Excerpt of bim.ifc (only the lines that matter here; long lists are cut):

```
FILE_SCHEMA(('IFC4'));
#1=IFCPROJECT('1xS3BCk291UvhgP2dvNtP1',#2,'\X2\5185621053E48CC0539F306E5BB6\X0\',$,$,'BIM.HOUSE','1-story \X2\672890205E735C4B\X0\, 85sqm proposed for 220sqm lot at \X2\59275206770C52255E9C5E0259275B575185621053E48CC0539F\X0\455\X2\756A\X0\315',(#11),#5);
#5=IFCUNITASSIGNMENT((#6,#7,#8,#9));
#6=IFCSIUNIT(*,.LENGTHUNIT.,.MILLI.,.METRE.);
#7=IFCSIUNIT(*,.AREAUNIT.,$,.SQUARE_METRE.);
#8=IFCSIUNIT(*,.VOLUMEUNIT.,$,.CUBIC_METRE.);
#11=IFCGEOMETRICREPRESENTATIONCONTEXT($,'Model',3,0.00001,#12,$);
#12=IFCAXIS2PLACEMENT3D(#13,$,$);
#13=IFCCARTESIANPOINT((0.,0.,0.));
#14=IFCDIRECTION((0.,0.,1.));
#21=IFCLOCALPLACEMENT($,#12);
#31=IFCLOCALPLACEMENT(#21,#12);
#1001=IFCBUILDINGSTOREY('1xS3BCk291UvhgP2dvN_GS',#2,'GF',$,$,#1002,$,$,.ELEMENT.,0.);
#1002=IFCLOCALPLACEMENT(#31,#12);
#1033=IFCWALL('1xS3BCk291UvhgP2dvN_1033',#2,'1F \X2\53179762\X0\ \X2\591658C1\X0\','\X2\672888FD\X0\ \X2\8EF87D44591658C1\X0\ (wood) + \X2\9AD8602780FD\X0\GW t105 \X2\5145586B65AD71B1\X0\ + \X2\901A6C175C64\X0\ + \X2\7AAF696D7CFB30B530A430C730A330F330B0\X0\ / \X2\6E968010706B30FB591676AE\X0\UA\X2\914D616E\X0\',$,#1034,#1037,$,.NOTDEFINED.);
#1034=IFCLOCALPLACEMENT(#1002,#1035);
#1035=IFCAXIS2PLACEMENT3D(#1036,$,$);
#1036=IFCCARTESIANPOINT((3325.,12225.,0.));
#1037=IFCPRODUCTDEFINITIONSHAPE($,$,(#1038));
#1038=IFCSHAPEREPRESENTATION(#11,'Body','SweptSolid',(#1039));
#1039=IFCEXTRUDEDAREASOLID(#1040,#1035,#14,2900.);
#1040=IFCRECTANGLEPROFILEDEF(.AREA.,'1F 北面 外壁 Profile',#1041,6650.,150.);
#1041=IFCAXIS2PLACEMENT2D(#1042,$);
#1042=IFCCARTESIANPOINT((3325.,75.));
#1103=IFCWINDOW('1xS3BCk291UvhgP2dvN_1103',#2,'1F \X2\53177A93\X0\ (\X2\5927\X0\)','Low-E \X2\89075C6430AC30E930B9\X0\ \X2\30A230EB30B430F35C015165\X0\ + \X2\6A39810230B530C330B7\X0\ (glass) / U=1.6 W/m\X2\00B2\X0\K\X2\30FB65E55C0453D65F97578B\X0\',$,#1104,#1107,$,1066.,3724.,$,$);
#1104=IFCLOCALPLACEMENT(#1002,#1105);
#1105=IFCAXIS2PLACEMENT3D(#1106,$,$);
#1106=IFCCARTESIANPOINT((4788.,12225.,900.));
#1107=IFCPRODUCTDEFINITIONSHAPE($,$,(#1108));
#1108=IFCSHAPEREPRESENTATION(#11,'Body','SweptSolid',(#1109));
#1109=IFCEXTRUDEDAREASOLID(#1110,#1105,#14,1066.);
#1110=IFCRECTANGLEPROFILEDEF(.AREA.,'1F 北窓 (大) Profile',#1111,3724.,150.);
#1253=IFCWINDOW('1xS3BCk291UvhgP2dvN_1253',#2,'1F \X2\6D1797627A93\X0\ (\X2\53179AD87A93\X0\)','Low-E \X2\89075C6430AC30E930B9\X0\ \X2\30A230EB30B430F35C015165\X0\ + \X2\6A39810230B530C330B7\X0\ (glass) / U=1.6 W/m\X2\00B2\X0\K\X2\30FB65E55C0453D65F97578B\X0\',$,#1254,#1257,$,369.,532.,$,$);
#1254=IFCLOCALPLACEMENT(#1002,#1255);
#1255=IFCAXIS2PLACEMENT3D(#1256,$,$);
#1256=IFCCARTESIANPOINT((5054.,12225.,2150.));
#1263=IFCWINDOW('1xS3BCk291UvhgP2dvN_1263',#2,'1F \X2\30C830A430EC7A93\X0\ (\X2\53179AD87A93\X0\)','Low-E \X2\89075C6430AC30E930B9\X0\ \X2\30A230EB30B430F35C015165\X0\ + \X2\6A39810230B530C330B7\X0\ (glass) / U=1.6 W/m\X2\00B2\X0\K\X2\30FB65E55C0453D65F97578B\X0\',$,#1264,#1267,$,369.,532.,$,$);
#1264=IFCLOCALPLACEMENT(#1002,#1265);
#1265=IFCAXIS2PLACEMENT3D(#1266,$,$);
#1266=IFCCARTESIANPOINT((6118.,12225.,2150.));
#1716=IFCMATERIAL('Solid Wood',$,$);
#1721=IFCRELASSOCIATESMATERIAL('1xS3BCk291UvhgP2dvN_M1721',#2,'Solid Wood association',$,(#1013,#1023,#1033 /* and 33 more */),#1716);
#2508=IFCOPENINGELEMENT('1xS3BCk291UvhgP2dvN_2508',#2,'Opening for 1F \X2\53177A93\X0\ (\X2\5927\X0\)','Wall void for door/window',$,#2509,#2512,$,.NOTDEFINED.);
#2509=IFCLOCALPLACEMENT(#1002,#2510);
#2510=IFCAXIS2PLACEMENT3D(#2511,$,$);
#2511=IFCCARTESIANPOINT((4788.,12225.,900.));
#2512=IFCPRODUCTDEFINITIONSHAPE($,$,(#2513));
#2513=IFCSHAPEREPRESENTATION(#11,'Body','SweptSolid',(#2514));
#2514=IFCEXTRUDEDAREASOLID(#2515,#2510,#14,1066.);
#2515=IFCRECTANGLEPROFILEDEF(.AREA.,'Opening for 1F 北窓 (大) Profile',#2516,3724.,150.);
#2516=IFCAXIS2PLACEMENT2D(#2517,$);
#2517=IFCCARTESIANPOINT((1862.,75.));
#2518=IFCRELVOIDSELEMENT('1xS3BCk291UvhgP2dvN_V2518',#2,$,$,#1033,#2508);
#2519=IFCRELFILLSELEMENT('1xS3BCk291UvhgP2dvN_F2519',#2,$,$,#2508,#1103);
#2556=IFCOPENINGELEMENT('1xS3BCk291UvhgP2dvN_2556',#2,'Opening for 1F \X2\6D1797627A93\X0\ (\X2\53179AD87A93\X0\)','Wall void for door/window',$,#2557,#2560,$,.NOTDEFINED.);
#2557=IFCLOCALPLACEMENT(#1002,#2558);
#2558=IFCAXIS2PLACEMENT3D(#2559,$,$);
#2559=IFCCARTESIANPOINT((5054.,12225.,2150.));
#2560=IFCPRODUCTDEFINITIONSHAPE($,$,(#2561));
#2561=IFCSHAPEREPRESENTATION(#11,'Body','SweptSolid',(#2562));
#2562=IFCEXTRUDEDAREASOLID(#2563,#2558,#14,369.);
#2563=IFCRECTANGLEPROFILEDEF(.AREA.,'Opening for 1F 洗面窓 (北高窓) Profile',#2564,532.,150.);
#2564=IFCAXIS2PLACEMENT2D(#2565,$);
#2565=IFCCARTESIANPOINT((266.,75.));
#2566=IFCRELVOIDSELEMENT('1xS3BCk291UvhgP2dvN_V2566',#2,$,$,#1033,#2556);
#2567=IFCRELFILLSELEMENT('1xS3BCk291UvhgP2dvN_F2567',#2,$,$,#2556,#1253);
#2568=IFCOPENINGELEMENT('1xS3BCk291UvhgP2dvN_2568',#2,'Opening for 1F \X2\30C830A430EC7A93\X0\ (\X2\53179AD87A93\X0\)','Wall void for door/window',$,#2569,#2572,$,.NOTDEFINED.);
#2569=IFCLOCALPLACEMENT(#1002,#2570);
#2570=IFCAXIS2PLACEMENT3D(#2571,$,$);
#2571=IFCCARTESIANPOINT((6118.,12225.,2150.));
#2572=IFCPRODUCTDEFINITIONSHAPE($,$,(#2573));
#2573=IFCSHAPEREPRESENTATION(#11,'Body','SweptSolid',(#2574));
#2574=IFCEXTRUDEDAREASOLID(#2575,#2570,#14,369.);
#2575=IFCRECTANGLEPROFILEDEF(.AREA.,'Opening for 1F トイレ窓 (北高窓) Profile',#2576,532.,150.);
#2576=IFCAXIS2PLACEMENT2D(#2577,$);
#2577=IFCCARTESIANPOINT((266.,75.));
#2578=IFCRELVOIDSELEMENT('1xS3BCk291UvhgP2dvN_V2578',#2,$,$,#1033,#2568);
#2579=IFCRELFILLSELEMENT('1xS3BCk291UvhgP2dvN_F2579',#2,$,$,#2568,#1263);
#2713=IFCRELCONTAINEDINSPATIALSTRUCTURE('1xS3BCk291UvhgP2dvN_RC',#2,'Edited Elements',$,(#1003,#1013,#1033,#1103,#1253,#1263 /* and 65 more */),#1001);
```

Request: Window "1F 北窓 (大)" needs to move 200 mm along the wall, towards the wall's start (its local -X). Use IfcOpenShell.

```python
import ifcopenshell
import ifcopenshell.api.geometry
import ifcopenshell.util.placement
import ifcopenshell.util.unit

model = ifcopenshell.open("bim.ifc")
unit_scale = ifcopenshell.util.unit.calculate_unit_scale(model)

window = model.by_id(1103)
opening = window.FillsVoids[0].RelatingOpeningElement
wall = opening.VoidsElements[0].RelatingBuildingElement

wall_matrix = ifcopenshell.util.placement.get_local_placement(wall.ObjectPlacement)
shift = wall_matrix[:3, 0] * -0.2 / unit_scale
before = ifcopenshell.util.placement.get_local_placement(window.ObjectPlacement)[:3, 3].copy()

# The window is not placed relative to its opening, so move both.
for product in (opening, window):
    matrix = ifcopenshell.util.placement.get_local_placement(product.ObjectPlacement)
    matrix[:3, 3] += shift
    ifcopenshell.api.geometry.edit_object_placement(model, product=product, matrix=matrix, is_si=False)

after = ifcopenshell.util.placement.get_local_placement(window.ObjectPlacement)[:3, 3]
print("window moved by", (after - before).round(3) + 0.0)

model.write("bim_updated.ifc")
```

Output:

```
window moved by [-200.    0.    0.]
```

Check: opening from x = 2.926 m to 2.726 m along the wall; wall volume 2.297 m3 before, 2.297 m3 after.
